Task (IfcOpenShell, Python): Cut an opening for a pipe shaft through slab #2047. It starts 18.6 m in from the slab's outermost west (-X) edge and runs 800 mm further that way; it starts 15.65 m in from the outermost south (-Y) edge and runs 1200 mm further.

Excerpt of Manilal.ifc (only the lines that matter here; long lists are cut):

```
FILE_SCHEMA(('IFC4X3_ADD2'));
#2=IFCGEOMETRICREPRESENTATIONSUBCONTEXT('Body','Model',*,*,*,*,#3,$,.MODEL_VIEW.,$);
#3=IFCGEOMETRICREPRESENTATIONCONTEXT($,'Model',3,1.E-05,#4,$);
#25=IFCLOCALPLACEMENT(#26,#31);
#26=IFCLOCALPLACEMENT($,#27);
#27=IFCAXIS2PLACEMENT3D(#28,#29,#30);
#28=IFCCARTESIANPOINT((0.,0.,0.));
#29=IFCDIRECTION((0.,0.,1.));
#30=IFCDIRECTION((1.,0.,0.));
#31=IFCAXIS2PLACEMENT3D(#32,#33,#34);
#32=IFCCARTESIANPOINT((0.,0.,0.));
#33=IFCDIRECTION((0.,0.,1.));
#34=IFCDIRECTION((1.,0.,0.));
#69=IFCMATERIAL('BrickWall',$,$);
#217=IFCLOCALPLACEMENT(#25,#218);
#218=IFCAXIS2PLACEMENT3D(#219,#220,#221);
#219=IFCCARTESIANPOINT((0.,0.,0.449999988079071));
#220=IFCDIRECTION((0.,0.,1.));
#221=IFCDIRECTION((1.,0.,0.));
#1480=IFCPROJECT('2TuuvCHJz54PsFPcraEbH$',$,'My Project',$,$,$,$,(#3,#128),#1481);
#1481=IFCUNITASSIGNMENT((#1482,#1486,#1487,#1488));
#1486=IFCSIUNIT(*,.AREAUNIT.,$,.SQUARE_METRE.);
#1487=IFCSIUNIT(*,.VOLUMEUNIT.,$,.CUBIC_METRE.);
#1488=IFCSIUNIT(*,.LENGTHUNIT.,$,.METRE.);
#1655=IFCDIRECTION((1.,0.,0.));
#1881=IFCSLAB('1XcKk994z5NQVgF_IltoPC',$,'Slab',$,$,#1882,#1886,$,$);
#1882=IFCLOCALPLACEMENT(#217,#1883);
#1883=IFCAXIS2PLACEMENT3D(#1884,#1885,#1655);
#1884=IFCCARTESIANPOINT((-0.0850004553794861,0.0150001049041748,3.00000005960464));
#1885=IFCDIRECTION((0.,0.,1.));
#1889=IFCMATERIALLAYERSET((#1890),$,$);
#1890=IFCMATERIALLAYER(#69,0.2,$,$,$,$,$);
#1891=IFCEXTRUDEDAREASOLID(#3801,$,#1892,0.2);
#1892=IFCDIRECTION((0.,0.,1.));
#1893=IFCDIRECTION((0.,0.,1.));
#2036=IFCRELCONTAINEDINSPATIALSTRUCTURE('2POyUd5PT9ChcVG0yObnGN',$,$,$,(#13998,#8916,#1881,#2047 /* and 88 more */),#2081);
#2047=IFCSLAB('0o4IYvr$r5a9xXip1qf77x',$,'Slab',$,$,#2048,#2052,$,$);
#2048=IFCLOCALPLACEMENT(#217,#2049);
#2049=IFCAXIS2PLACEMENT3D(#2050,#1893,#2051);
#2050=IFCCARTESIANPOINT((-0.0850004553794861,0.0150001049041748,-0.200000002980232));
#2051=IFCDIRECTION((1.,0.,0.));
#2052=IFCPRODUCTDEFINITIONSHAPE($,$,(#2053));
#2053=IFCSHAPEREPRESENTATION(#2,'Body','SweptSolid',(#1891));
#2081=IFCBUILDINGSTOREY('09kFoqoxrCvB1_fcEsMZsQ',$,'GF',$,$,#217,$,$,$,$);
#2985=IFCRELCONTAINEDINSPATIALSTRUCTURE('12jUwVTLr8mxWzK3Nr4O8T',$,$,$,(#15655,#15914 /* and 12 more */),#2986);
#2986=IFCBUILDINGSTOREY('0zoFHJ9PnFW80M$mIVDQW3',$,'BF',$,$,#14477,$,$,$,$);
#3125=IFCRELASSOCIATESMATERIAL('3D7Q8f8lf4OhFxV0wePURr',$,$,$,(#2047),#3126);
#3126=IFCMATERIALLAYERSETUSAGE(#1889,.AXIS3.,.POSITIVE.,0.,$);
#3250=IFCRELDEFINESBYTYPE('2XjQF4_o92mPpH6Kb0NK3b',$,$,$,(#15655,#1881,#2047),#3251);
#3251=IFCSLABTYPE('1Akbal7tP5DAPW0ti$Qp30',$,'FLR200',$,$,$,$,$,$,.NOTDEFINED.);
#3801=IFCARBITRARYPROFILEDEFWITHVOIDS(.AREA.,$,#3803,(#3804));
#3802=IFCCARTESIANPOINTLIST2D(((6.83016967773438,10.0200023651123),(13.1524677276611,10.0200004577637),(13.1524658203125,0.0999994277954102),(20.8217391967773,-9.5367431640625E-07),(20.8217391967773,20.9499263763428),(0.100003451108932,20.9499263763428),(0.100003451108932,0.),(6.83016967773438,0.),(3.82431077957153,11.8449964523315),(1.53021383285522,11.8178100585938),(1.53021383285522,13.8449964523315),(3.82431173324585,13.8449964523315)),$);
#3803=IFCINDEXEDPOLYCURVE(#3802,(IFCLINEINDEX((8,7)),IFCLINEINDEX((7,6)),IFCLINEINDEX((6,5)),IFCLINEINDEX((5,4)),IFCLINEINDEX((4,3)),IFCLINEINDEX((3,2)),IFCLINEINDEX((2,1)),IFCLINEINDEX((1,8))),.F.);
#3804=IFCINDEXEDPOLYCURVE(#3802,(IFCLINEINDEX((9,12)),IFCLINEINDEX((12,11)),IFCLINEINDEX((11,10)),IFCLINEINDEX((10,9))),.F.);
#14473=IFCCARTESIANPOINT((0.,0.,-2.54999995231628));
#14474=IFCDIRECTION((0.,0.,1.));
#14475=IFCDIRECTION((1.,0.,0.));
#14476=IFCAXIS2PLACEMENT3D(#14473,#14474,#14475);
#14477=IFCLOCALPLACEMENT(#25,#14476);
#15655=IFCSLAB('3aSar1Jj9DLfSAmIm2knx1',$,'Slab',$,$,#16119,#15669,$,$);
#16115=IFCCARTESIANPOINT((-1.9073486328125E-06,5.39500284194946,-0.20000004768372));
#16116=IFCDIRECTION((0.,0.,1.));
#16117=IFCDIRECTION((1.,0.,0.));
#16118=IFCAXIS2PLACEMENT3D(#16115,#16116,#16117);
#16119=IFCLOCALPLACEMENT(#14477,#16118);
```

```python
import numpy as np
import ifcopenshell
import ifcopenshell.api.feature
import ifcopenshell.api.geometry
import ifcopenshell.api.root
import ifcopenshell.geom
import ifcopenshell.util.placement
import ifcopenshell.util.representation
import ifcopenshell.util.shape
import ifcopenshell.util.unit

model = ifcopenshell.open("Manilal.ifc")
unit_scale = ifcopenshell.util.unit.calculate_unit_scale(model)
settings = ifcopenshell.geom.settings()


def volume(element):
    """Net volume in cubic metres, openings subtracted."""
    shape = ifcopenshell.geom.create_shape(settings, element)
    return ifcopenshell.util.shape.get_volume(shape.geometry)


slab = model.by_guid("0o4IYvr$r5a9xXip1qf77x")
before = volume(slab)

# Extent in the slab's own axes, in metres. The edges named are its -X and -Y sides.
slab_shape = ifcopenshell.geom.create_shape(settings, slab)
vertices = ifcopenshell.util.shape.get_vertices(slab_shape.geometry)
x_min, y_min, bottom = vertices.min(axis=0)
top = vertices[:, 2].max()

opening = ifcopenshell.api.root.create_entity(model, ifc_class="IfcOpeningElement", name="Pipe shaft opening", predefined_type="OPENING")
context = ifcopenshell.util.representation.get_context(model, "Model", "Body", "MODEL_VIEW")
width, depth = 0.8, 1.2
outline = [(0.0, 0.0), (width, 0.0), (width, depth), (0.0, depth), (0.0, 0.0)]
# Overshoot both faces by 50 mm so the cut is clean.
shape = ifcopenshell.api.geometry.add_slab_representation(
    model, context=context, depth=top - bottom + 0.1, polyline=outline
)
ifcopenshell.api.geometry.assign_representation(model, product=opening, representation=shape)

matrix = ifcopenshell.util.placement.get_local_placement(slab.ObjectPlacement)
matrix[:, 3] = matrix @ np.append(np.array([x_min + 18.6, y_min + 15.65, bottom - 0.05]) / unit_scale, 1.0)
ifcopenshell.api.geometry.edit_object_placement(model, product=opening, matrix=matrix, is_si=False)
ifcopenshell.api.feature.add_feature(model, feature=opening, element=slab)

after = volume(slab)

print(f"slab volume {before:.3f} -> {after:.3f} m3")

model.write("Manilal_updated.ifc")
```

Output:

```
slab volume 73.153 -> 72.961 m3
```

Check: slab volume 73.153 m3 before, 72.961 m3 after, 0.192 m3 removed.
